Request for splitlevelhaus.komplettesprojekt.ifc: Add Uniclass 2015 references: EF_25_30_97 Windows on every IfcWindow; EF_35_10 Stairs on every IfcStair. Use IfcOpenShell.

First a look at what the model holds.

```python
import ifcopenshell

model = ifcopenshell.open("splitlevelhaus.komplettesprojekt.ifc")
print(model.schema)
print("classifications:", [c.Name for c in model.by_type("IfcClassification")])
for ifc_class in ("IfcDoor", "IfcRoof", "IfcStair", "IfcWall", "IfcWindow"):
    print(ifc_class, len(model.by_type(ifc_class)))
```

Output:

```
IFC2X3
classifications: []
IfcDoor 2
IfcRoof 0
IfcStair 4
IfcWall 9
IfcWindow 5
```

```python
import ifcopenshell
import ifcopenshell.api.classification

model = ifcopenshell.open("splitlevelhaus.komplettesprojekt.ifc")

# IFC2X3 requires Source and Edition and has no link from the project to the system.
system = model.create_entity("IfcClassification", Source="NBS", Edition="2015", Name="Uniclass 2015")

codes = {
    "IfcWindow": ("EF_25_30_97", "Windows"),
    "IfcStair": ("EF_35_10", "Stairs"),
}
for ifc_class, (code, name) in codes.items():
    products = model.by_type(ifc_class)
    ifcopenshell.api.classification.add_reference(
        model, products=products, classification=system, identification=code, name=name
    )
    print(code, len(products))

model.write("splitlevelhaus.komplettesprojekt_v2.ifc")
```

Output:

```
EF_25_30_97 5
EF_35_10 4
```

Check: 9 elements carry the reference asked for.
